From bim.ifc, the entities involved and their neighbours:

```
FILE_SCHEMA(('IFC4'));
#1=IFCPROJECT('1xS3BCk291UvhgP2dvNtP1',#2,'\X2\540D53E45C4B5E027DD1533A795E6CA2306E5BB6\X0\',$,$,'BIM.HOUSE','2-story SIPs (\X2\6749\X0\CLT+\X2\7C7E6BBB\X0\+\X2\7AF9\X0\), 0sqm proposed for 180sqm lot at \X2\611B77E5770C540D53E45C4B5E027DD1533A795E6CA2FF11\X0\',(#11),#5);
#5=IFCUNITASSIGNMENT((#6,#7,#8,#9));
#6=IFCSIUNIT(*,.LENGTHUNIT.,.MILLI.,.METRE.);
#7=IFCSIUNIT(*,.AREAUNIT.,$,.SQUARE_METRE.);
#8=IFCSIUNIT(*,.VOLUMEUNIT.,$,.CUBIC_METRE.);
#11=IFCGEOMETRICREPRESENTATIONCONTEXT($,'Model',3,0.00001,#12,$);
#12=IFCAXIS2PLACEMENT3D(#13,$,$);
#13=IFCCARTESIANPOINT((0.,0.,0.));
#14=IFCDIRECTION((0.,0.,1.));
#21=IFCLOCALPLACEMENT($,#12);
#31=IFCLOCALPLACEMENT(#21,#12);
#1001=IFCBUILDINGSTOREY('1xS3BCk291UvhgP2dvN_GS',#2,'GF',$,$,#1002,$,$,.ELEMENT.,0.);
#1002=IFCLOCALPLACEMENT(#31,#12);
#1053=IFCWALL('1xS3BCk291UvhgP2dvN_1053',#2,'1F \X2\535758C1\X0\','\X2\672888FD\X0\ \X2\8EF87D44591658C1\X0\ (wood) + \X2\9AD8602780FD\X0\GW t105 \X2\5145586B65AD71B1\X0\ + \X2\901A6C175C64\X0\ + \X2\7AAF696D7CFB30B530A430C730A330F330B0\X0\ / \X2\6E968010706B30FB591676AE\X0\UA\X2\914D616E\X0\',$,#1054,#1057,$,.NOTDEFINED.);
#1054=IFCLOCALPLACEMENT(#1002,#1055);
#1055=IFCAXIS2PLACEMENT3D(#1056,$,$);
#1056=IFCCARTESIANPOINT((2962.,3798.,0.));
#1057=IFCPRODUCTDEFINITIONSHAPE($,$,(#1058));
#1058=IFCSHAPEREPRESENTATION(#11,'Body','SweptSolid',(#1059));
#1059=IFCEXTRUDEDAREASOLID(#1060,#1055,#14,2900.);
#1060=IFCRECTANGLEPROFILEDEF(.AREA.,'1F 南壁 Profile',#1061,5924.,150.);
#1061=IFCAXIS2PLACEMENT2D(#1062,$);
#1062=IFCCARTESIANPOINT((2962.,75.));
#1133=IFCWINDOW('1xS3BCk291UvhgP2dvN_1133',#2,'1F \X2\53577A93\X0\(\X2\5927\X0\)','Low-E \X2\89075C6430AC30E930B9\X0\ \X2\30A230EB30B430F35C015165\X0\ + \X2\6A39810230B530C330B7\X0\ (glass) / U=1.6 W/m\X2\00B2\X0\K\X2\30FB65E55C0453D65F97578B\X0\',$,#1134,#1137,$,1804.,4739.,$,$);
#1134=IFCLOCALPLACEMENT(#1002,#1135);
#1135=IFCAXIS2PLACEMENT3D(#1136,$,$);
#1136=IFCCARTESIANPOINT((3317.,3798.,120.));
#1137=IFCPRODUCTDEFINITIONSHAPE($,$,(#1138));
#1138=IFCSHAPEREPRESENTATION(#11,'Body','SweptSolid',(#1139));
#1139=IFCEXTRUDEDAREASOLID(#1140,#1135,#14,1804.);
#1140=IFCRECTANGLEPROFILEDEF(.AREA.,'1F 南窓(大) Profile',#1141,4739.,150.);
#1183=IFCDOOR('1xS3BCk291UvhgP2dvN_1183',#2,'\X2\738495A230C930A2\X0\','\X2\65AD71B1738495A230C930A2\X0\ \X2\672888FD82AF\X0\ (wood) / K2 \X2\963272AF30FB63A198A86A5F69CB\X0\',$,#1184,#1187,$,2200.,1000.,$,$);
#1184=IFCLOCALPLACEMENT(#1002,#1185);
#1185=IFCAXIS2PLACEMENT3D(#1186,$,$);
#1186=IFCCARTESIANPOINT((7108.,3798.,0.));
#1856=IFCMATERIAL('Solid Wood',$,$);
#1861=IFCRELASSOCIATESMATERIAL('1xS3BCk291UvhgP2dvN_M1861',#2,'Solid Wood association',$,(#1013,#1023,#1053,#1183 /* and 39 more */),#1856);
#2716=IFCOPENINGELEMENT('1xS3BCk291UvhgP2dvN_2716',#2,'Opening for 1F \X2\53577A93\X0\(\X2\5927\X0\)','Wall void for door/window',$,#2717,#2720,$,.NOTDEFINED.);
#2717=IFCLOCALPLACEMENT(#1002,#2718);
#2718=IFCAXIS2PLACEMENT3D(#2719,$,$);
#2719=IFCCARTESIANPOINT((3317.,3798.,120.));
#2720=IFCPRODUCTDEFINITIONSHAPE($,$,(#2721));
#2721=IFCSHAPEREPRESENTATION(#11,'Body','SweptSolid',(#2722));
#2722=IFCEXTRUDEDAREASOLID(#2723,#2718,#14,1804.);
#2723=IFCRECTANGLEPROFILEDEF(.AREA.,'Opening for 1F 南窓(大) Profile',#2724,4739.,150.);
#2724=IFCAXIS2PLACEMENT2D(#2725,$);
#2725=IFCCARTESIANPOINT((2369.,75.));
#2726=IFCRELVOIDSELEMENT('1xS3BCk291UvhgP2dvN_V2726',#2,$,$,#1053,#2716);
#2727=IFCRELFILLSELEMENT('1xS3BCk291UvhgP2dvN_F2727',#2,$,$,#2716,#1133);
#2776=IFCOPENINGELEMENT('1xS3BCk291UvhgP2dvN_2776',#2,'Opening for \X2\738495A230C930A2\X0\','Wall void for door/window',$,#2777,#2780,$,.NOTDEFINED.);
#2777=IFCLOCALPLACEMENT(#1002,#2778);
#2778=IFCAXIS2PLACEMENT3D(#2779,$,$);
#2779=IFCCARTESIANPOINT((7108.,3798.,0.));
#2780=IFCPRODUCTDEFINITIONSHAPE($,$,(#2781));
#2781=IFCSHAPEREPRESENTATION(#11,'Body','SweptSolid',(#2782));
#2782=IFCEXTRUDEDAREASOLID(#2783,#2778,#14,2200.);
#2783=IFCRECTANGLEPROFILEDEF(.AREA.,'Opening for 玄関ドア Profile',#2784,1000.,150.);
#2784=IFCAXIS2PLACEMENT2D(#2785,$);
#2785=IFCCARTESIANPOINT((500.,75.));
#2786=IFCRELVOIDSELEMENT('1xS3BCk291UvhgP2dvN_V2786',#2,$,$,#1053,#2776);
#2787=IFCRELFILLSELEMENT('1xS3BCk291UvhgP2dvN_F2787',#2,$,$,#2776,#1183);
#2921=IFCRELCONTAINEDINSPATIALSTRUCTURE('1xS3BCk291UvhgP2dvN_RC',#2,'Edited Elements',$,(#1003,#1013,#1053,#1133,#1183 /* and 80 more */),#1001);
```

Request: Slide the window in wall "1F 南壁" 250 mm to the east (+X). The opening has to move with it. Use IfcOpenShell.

```python
import ifcopenshell
import ifcopenshell.api.geometry
import ifcopenshell.util.placement
import ifcopenshell.util.unit

model = ifcopenshell.open("bim.ifc")
unit_scale = ifcopenshell.util.unit.calculate_unit_scale(model)

window = model.by_id(1133)
opening = window.FillsVoids[0].RelatingOpeningElement
wall = opening.VoidsElements[0].RelatingBuildingElement

wall_matrix = ifcopenshell.util.placement.get_local_placement(wall.ObjectPlacement)
shift = wall_matrix[:3, 0] * 0.25 / unit_scale
before = ifcopenshell.util.placement.get_local_placement(window.ObjectPlacement)[:3, 3].copy()

# The window is not placed relative to its opening, so move both.
for product in (opening, window):
    matrix = ifcopenshell.util.placement.get_local_placement(product.ObjectPlacement)
    matrix[:3, 3] += shift
    ifcopenshell.api.geometry.edit_object_placement(model, product=product, matrix=matrix, is_si=False)

after = ifcopenshell.util.placement.get_local_placement(window.ObjectPlacement)[:3, 3]
print("window moved by", (after - before).round(3) + 0.0)

model.write("bim_updated.ifc")
```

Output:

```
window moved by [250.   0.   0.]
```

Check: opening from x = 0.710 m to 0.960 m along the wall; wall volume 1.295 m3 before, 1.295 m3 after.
